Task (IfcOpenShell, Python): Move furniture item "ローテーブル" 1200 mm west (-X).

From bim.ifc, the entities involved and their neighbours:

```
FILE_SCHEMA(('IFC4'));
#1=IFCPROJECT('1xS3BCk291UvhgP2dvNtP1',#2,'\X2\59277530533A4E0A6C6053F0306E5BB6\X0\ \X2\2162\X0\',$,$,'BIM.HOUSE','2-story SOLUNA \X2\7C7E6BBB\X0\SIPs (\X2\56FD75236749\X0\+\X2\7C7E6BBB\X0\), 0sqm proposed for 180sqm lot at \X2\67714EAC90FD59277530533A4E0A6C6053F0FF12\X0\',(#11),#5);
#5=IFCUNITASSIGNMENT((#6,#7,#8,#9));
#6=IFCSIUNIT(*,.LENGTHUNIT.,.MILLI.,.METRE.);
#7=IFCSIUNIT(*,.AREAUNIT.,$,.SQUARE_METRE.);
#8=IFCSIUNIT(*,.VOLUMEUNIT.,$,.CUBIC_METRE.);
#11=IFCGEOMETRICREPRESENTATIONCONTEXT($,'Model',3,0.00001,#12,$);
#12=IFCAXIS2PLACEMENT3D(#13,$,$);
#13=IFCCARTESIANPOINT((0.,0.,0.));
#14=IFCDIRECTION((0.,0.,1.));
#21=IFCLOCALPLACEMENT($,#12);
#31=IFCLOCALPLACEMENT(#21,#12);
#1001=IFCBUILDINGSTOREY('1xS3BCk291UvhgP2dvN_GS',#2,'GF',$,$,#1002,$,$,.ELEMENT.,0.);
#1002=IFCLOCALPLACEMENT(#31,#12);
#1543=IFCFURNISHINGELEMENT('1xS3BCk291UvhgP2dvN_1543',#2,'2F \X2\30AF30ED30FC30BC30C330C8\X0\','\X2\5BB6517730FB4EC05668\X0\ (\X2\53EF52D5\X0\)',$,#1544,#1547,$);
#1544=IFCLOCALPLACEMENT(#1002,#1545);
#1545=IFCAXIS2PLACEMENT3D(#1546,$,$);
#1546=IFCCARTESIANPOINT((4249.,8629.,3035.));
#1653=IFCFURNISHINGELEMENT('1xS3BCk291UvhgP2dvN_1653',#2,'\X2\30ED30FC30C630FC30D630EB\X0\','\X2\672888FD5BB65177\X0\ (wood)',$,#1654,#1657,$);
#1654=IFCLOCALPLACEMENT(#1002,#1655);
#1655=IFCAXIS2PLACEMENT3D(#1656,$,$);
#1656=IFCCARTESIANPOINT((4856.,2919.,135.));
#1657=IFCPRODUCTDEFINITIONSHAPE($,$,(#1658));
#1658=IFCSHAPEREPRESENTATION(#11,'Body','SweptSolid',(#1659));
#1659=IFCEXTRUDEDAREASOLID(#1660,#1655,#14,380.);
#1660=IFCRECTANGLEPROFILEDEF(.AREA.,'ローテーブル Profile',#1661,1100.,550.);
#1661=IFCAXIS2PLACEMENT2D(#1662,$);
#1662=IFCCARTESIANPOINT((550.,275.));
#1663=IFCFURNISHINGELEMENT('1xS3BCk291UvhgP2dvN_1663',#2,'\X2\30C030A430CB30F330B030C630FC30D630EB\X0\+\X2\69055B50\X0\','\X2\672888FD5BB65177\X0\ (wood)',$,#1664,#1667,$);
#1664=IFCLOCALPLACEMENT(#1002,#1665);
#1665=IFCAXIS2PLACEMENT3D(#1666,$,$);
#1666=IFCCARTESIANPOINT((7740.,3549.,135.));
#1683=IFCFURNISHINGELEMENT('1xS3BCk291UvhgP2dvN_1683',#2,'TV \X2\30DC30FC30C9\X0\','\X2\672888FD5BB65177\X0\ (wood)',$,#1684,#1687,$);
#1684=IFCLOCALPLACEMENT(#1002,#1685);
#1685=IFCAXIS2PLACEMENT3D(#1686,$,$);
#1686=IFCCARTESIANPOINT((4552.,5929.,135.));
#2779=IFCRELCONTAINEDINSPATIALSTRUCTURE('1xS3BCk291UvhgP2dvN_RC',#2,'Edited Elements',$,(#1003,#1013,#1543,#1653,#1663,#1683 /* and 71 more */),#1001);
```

```python
import ifcopenshell
import ifcopenshell.api.geometry
import ifcopenshell.util.placement
import ifcopenshell.util.unit

model = ifcopenshell.open("bim.ifc")
unit_scale = ifcopenshell.util.unit.calculate_unit_scale(model)

item = model.by_id(1653)
matrix = ifcopenshell.util.placement.get_local_placement(item.ObjectPlacement)
matrix[0, 3] -= 1.2 / unit_scale
ifcopenshell.api.geometry.edit_object_placement(model, product=item, matrix=matrix, is_si=False)

print(ifcopenshell.util.placement.get_local_placement(item.ObjectPlacement).round(3) + 0.0)

model.write("bim_edited.ifc")
```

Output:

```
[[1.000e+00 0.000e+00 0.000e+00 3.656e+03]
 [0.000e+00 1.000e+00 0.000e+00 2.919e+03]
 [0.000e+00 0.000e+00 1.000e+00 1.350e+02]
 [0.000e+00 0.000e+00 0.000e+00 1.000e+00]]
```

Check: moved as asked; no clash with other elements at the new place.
